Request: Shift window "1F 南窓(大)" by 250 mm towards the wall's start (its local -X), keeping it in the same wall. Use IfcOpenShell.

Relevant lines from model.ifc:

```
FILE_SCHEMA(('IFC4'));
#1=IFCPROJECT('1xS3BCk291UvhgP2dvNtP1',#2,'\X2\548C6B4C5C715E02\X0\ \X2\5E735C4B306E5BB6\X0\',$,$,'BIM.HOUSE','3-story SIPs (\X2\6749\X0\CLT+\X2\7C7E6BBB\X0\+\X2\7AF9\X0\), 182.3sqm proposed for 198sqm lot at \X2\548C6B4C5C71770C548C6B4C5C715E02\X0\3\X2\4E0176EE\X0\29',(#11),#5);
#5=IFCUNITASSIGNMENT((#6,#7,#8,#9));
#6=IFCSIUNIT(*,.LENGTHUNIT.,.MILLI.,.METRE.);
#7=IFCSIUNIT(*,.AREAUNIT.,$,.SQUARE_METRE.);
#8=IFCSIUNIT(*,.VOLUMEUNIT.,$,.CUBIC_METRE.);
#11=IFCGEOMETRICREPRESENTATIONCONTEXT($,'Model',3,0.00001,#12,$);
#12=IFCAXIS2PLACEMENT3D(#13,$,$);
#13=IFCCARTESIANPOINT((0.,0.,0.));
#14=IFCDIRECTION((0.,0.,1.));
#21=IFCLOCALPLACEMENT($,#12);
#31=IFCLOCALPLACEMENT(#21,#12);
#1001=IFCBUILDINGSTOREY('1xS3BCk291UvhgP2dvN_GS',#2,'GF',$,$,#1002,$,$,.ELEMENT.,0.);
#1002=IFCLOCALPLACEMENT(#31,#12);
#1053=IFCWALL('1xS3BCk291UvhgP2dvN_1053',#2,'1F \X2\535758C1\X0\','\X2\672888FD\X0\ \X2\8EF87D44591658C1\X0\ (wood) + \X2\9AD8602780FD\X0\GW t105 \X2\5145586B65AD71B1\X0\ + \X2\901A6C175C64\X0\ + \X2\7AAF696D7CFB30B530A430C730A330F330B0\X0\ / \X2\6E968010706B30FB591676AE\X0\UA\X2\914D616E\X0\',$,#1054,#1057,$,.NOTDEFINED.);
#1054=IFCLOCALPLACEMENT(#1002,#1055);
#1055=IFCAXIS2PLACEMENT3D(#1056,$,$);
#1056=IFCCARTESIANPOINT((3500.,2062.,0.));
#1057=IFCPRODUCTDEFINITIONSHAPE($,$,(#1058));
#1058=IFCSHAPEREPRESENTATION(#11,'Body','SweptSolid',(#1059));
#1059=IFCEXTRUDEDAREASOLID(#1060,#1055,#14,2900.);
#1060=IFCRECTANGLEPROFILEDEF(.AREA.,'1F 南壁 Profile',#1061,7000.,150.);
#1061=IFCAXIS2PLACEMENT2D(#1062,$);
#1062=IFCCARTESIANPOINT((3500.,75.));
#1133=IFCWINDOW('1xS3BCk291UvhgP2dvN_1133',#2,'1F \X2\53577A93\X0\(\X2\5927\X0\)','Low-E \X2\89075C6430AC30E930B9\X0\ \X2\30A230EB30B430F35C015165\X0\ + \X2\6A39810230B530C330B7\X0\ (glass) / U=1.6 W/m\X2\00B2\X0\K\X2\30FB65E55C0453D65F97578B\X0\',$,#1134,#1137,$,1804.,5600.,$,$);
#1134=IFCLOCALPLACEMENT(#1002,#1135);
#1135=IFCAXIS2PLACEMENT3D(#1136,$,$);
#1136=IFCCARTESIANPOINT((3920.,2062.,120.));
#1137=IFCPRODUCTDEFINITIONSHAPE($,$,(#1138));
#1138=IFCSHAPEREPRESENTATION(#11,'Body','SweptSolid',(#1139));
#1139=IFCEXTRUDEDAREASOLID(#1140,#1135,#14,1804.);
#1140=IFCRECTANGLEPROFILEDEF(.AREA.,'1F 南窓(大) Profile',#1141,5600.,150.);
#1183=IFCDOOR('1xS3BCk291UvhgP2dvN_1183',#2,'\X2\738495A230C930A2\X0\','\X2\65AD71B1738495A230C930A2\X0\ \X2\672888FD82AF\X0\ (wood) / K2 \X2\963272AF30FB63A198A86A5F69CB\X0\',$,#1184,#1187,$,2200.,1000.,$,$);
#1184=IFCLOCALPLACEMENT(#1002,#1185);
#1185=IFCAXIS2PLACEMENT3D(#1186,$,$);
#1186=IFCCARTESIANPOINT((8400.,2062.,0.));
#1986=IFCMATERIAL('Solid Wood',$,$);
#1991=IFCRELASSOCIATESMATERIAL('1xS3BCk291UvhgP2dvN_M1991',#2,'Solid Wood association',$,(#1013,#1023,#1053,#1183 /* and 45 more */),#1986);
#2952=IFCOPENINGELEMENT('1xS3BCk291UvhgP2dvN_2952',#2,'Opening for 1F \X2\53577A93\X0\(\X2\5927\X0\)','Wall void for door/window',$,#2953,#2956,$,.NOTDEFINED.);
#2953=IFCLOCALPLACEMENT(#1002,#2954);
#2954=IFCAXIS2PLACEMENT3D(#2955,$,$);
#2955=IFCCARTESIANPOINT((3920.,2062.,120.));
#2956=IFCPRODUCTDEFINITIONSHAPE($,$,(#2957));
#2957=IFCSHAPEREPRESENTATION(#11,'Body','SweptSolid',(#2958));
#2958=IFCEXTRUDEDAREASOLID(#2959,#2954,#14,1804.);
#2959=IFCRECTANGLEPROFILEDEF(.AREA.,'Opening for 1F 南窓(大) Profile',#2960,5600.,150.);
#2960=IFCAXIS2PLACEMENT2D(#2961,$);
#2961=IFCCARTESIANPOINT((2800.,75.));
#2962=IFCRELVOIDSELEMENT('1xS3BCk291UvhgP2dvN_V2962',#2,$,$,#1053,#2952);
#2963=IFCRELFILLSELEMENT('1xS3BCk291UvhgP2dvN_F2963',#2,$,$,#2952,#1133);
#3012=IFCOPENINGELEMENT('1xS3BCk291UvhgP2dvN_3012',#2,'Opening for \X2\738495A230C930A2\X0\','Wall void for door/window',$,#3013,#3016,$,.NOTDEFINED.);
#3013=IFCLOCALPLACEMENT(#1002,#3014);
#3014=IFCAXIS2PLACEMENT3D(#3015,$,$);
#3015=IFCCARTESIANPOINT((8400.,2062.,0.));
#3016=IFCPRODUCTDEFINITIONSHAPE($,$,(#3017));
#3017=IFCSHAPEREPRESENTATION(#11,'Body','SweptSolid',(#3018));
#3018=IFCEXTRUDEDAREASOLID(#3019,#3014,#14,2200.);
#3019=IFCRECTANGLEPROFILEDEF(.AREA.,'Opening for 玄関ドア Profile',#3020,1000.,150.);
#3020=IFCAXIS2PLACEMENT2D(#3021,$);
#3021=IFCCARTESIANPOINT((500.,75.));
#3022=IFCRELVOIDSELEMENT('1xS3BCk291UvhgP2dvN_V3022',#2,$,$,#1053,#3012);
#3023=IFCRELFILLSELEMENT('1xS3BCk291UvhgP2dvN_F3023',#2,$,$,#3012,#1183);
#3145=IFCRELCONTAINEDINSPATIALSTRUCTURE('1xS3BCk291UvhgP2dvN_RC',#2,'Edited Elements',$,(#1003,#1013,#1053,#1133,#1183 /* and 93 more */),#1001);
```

```python
import ifcopenshell
import ifcopenshell.api.geometry
import ifcopenshell.util.placement
import ifcopenshell.util.unit

model = ifcopenshell.open("model.ifc")
unit_scale = ifcopenshell.util.unit.calculate_unit_scale(model)

window = model.by_guid("1xS3BCk291UvhgP2dvN_1133")
opening = window.FillsVoids[0].RelatingOpeningElement
wall = opening.VoidsElements[0].RelatingBuildingElement

wall_matrix = ifcopenshell.util.placement.get_local_placement(wall.ObjectPlacement)
shift = wall_matrix[:3, 0] * -0.25 / unit_scale
before = ifcopenshell.util.placement.get_local_placement(window.ObjectPlacement)[:3, 3].copy()

# The window is not placed relative to its opening, so move both.
for product in (opening, window):
    matrix = ifcopenshell.util.placement.get_local_placement(product.ObjectPlacement)
    matrix[:3, 3] += shift
    ifcopenshell.api.geometry.edit_object_placement(model, product=product, matrix=matrix, is_si=False)

after = ifcopenshell.util.placement.get_local_placement(window.ObjectPlacement)[:3, 3]
print("window moved by", (after - before).round(3) + 0.0)

model.write("model_rev.ifc")
```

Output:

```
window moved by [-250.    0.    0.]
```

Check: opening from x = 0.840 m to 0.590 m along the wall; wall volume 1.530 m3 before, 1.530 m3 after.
